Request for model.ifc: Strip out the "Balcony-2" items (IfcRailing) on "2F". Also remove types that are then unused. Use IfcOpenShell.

First a look at what the model holds.

```python
import ifcopenshell
import ifcopenshell.util.element

model = ifcopenshell.open("model.ifc")
print(model.schema)
storey = next(s for s in model.by_type("IfcBuildingStorey") if s.Name == "2F")
railings = [e for e in ifcopenshell.util.element.get_decomposition(storey) if e.is_a("IfcRailing")]
seen = {}
for e in railings:
    element_type = ifcopenshell.util.element.get_type(e)
    name = element_type.Name if element_type not in (None, e) else None
    seen[name] = seen.get(name, 0) + 1
for name, count in sorted(seen.items(), key=str):
    print(count, "x", name)
```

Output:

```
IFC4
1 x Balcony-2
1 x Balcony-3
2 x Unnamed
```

```python
import ifcopenshell
import ifcopenshell.api.root
import ifcopenshell.util.element

model = ifcopenshell.open("model.ifc")

storey = next(s for s in model.by_type("IfcBuildingStorey") if s.Name == "2F")
railings = [e for e in ifcopenshell.util.element.get_decomposition(storey) if e.is_a("IfcRailing")]
targets = [e for e in railings if (t := ifcopenshell.util.element.get_type(e)) not in (None, e) and t.Name == "Balcony-2"]
types = {ifcopenshell.util.element.get_type(e) for e in targets} - {None, *targets}

for e in targets:
    ifcopenshell.api.root.remove_product(model, product=e)
print(len(targets), "removed")

unused = [t for t in types if not ifcopenshell.util.element.get_types(t)]
for t in unused:
    ifcopenshell.api.root.remove_product(model, product=t)
print(len(unused), "unused types removed")

model.write("model_rev.ifc")
```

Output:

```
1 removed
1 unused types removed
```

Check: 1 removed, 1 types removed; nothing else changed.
